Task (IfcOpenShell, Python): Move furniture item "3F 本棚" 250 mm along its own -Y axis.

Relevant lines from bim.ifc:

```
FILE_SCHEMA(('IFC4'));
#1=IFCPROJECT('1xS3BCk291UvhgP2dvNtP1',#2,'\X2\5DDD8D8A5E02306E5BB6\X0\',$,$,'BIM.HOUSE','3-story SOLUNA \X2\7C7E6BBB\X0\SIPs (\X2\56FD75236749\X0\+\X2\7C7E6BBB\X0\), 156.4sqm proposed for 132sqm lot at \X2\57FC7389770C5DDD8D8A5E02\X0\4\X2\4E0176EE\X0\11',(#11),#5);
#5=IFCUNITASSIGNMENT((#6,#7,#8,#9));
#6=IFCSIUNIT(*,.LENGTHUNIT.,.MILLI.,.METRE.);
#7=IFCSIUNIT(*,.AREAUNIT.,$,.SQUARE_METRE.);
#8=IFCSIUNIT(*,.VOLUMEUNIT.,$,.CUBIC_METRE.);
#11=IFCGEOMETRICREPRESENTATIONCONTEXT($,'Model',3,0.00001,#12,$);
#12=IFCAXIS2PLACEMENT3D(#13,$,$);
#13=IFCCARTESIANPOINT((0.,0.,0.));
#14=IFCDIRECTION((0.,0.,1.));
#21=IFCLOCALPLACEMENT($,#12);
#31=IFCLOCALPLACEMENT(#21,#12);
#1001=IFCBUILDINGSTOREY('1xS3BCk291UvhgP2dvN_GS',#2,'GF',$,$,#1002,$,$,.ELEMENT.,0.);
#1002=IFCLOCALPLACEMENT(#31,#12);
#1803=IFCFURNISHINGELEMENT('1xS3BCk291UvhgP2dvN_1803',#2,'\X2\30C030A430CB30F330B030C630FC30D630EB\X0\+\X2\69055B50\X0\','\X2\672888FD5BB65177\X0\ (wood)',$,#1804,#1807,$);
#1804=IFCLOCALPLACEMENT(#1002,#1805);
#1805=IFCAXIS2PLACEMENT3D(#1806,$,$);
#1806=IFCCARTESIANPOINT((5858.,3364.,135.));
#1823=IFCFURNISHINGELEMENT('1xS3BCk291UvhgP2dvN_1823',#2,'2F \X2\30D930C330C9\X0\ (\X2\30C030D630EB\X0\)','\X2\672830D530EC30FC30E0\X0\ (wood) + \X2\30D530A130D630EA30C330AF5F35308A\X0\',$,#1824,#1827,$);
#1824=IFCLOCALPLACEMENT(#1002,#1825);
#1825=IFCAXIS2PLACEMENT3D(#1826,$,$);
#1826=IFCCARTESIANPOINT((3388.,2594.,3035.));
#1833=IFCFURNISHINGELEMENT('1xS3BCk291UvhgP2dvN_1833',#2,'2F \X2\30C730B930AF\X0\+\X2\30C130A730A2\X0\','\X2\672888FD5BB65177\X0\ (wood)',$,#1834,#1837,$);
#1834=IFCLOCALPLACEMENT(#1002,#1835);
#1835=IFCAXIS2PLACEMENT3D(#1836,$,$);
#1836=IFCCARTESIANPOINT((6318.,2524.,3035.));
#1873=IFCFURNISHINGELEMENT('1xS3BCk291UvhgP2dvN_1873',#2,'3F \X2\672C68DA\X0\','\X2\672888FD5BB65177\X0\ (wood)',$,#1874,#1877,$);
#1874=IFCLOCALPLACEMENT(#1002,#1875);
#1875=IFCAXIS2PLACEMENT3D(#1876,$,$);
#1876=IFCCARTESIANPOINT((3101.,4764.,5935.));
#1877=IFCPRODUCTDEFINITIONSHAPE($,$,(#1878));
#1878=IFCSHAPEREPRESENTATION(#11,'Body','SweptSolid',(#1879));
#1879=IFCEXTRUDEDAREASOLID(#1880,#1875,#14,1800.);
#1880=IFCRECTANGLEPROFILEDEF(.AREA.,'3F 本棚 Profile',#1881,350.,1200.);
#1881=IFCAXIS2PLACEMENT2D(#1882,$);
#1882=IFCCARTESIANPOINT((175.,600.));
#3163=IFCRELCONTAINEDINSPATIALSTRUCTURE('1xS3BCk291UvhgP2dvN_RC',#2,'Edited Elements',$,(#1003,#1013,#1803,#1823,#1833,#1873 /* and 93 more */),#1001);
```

```python
import ifcopenshell
import ifcopenshell.api.geometry
import ifcopenshell.util.placement
import ifcopenshell.util.unit

model = ifcopenshell.open("bim.ifc")
unit_scale = ifcopenshell.util.unit.calculate_unit_scale(model)

item = model.by_guid("1xS3BCk291UvhgP2dvN_1873")
matrix = ifcopenshell.util.placement.get_local_placement(item.ObjectPlacement)
matrix[:3, 3] -= matrix[:3, 1] * 0.25 / unit_scale
ifcopenshell.api.geometry.edit_object_placement(model, product=item, matrix=matrix, is_si=False)

print(ifcopenshell.util.placement.get_local_placement(item.ObjectPlacement).round(3) + 0.0)

model.write("bim_edited.ifc")
```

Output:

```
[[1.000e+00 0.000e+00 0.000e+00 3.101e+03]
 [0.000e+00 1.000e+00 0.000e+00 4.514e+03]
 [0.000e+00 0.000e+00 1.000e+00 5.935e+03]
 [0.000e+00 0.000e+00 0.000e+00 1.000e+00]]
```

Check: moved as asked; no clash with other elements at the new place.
